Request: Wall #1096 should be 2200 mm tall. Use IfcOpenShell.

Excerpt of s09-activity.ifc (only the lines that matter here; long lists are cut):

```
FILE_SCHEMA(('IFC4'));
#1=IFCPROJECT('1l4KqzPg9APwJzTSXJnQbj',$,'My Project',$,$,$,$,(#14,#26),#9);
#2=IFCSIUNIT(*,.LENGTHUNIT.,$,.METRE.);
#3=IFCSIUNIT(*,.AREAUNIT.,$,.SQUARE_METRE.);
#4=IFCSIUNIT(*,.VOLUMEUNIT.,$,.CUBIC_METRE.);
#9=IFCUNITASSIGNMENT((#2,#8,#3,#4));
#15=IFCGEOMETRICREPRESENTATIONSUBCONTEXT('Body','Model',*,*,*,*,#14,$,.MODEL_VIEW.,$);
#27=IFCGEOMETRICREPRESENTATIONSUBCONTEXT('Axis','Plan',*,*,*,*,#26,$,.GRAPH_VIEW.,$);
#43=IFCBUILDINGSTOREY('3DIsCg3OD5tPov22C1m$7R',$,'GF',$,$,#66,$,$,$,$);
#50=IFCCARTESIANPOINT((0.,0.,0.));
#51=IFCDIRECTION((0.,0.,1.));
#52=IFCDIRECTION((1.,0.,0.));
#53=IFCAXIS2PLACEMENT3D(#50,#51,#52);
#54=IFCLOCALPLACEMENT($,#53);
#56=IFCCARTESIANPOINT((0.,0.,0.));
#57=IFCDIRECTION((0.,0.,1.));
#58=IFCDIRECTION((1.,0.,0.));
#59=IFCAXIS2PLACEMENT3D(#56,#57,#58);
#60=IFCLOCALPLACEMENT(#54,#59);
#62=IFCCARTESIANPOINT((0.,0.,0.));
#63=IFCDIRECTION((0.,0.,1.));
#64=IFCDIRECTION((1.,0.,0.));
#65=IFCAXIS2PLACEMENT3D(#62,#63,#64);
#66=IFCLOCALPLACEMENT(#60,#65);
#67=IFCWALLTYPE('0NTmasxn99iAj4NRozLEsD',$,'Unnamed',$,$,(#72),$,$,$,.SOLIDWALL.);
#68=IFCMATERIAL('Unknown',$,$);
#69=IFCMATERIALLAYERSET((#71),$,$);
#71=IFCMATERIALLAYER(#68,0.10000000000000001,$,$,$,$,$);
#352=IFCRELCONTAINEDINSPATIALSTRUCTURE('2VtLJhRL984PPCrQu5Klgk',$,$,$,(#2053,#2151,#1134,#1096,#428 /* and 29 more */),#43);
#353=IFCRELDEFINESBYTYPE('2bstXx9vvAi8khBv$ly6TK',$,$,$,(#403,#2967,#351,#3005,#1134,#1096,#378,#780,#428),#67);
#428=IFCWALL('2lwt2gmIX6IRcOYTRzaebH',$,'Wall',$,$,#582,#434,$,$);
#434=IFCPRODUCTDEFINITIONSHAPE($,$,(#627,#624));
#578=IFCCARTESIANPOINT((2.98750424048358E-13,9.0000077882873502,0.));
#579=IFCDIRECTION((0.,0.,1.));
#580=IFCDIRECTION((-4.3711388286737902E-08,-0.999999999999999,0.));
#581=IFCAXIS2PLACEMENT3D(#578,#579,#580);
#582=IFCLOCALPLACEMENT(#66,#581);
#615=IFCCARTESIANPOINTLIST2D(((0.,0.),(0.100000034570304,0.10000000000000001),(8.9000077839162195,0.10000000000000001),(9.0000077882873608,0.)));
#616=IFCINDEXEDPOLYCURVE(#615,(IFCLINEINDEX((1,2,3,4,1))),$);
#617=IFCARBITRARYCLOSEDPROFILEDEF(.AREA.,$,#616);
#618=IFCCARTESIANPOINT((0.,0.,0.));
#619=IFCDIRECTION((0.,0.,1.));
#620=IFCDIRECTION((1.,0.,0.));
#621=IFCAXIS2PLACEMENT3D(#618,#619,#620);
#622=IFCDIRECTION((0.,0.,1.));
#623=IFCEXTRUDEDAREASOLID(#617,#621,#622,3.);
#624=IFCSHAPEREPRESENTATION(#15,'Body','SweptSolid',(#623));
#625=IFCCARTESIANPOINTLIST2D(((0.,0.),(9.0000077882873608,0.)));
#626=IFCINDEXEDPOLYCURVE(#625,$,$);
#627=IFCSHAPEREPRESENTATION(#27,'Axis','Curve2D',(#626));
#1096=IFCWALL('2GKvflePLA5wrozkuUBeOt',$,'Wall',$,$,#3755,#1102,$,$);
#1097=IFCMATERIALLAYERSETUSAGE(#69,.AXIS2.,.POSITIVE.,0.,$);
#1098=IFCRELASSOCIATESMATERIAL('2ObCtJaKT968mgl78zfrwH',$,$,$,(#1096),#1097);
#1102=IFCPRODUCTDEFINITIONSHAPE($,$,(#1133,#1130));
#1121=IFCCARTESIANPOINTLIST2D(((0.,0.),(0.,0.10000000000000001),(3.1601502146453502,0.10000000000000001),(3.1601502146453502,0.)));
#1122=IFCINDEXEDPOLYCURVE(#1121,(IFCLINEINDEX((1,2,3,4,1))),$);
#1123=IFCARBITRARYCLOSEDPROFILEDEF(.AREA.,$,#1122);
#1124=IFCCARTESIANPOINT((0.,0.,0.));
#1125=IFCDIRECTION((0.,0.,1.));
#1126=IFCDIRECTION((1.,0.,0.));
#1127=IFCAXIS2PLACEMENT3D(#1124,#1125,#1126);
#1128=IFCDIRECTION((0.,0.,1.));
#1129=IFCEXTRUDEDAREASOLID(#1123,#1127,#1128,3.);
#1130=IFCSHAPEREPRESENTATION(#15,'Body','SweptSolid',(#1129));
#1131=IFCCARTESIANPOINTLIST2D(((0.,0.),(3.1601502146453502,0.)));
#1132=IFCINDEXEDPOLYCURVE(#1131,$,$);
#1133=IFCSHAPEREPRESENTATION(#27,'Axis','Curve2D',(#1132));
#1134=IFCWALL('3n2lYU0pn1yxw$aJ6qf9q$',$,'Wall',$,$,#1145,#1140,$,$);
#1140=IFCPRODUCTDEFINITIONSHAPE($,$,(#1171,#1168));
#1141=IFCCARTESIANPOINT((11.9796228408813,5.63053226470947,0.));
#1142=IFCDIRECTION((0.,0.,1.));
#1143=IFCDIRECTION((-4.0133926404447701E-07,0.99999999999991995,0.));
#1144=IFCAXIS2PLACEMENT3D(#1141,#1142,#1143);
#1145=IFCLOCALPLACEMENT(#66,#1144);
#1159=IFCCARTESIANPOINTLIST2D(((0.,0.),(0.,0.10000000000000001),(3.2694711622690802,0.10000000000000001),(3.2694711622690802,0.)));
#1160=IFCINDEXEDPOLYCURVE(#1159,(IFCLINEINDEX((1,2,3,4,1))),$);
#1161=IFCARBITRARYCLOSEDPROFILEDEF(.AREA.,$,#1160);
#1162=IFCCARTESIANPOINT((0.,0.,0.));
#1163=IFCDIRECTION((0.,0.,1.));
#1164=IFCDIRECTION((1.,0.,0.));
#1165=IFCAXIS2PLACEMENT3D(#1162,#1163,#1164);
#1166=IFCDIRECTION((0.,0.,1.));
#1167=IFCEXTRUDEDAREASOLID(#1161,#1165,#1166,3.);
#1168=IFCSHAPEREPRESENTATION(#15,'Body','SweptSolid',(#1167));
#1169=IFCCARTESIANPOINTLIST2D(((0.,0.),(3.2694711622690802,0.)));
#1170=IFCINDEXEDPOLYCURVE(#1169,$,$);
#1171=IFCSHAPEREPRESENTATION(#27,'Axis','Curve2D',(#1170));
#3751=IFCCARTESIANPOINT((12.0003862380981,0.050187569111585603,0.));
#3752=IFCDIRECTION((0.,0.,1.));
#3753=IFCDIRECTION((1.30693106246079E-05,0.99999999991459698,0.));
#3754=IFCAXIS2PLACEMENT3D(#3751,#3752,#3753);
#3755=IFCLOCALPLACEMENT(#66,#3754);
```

```python
import ifcopenshell
import ifcopenshell.geom
import ifcopenshell.util.representation
import ifcopenshell.util.shape
import ifcopenshell.util.unit

model = ifcopenshell.open("s09-activity.ifc")
unit_scale = ifcopenshell.util.unit.calculate_unit_scale(model)
settings = ifcopenshell.geom.settings()


def volume(element):
    """Net volume in cubic metres, openings subtracted."""
    shape = ifcopenshell.geom.create_shape(settings, element)
    return ifcopenshell.util.shape.get_volume(shape.geometry)


wall = model.by_guid("2GKvflePLA5wrozkuUBeOt")
before = volume(wall)

body = ifcopenshell.util.representation.get_representation(wall, "Model", "Body")
solid = body.Items[0]
old_height = solid.Depth
solid.Depth = 2.2 / unit_scale
after = volume(wall)

print(f"height {old_height:g} -> {solid.Depth:g}, volume {before:.3f} -> {after:.3f} m3")

model.write("s09-activity_rev.ifc")
```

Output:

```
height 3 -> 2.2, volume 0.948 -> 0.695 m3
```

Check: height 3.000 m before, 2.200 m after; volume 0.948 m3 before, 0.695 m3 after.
